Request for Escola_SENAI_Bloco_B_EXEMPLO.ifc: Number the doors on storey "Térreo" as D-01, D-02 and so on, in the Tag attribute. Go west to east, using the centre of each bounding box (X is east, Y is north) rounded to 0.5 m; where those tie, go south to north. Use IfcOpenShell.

First a look at what the model holds.

```python
import ifcopenshell
import ifcopenshell.util.element
import ifcopenshell.util.placement

model = ifcopenshell.open("Escola_SENAI_Bloco_B_EXEMPLO.ifc")
print(model.schema)
storey = next(s for s in model.by_type("IfcBuildingStorey") if s.Name == "Térreo")
doors = [e for e in ifcopenshell.util.element.get_decomposition(storey) if e.is_a("IfcDoor")]
for e in sorted(doors, key=lambda e: e.id()):
    origin = ifcopenshell.util.placement.get_local_placement(e.ObjectPlacement)[:3, 3]
    print(e.id(), e.Tag, e.Name, origin.round(2) + 0.0, sep=" | ")
```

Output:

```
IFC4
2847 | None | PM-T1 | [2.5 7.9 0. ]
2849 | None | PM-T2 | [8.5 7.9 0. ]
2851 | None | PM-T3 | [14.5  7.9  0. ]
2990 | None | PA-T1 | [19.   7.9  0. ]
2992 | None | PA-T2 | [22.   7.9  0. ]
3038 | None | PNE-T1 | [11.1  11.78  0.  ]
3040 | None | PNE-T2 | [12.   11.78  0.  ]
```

```python
import ifcopenshell
import ifcopenshell.geom
import ifcopenshell.util.element
import ifcopenshell.util.shape

model = ifcopenshell.open("Escola_SENAI_Bloco_B_EXEMPLO.ifc")
settings = ifcopenshell.geom.settings()
settings.set("use-world-coords", True)


def centre(element):
    shape = ifcopenshell.geom.create_shape(settings, element)
    return ifcopenshell.util.shape.get_bbox_centroid(shape.geometry)


storey = next(s for s in model.by_type("IfcBuildingStorey") if s.Name == "Térreo")
doors = [e for e in ifcopenshell.util.element.get_decomposition(storey) if e.is_a("IfcDoor")]

# Insertion points can sit at a corner or the storey origin, so sort by the geometry (in metres).
centres = {e: centre(e) for e in doors}
doors.sort(key=lambda e: (round(centres[e][0] / 0.5), centres[e][1]))

for i, e in enumerate(doors, start=1):
    number = f"D-{i:02d}"
    e.Tag = number
    print(e.id(), number)

model.write("Escola_SENAI_Bloco_B_EXEMPLO_rev.ifc")
```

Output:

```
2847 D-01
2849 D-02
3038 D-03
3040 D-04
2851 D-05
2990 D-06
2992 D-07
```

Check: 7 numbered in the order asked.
